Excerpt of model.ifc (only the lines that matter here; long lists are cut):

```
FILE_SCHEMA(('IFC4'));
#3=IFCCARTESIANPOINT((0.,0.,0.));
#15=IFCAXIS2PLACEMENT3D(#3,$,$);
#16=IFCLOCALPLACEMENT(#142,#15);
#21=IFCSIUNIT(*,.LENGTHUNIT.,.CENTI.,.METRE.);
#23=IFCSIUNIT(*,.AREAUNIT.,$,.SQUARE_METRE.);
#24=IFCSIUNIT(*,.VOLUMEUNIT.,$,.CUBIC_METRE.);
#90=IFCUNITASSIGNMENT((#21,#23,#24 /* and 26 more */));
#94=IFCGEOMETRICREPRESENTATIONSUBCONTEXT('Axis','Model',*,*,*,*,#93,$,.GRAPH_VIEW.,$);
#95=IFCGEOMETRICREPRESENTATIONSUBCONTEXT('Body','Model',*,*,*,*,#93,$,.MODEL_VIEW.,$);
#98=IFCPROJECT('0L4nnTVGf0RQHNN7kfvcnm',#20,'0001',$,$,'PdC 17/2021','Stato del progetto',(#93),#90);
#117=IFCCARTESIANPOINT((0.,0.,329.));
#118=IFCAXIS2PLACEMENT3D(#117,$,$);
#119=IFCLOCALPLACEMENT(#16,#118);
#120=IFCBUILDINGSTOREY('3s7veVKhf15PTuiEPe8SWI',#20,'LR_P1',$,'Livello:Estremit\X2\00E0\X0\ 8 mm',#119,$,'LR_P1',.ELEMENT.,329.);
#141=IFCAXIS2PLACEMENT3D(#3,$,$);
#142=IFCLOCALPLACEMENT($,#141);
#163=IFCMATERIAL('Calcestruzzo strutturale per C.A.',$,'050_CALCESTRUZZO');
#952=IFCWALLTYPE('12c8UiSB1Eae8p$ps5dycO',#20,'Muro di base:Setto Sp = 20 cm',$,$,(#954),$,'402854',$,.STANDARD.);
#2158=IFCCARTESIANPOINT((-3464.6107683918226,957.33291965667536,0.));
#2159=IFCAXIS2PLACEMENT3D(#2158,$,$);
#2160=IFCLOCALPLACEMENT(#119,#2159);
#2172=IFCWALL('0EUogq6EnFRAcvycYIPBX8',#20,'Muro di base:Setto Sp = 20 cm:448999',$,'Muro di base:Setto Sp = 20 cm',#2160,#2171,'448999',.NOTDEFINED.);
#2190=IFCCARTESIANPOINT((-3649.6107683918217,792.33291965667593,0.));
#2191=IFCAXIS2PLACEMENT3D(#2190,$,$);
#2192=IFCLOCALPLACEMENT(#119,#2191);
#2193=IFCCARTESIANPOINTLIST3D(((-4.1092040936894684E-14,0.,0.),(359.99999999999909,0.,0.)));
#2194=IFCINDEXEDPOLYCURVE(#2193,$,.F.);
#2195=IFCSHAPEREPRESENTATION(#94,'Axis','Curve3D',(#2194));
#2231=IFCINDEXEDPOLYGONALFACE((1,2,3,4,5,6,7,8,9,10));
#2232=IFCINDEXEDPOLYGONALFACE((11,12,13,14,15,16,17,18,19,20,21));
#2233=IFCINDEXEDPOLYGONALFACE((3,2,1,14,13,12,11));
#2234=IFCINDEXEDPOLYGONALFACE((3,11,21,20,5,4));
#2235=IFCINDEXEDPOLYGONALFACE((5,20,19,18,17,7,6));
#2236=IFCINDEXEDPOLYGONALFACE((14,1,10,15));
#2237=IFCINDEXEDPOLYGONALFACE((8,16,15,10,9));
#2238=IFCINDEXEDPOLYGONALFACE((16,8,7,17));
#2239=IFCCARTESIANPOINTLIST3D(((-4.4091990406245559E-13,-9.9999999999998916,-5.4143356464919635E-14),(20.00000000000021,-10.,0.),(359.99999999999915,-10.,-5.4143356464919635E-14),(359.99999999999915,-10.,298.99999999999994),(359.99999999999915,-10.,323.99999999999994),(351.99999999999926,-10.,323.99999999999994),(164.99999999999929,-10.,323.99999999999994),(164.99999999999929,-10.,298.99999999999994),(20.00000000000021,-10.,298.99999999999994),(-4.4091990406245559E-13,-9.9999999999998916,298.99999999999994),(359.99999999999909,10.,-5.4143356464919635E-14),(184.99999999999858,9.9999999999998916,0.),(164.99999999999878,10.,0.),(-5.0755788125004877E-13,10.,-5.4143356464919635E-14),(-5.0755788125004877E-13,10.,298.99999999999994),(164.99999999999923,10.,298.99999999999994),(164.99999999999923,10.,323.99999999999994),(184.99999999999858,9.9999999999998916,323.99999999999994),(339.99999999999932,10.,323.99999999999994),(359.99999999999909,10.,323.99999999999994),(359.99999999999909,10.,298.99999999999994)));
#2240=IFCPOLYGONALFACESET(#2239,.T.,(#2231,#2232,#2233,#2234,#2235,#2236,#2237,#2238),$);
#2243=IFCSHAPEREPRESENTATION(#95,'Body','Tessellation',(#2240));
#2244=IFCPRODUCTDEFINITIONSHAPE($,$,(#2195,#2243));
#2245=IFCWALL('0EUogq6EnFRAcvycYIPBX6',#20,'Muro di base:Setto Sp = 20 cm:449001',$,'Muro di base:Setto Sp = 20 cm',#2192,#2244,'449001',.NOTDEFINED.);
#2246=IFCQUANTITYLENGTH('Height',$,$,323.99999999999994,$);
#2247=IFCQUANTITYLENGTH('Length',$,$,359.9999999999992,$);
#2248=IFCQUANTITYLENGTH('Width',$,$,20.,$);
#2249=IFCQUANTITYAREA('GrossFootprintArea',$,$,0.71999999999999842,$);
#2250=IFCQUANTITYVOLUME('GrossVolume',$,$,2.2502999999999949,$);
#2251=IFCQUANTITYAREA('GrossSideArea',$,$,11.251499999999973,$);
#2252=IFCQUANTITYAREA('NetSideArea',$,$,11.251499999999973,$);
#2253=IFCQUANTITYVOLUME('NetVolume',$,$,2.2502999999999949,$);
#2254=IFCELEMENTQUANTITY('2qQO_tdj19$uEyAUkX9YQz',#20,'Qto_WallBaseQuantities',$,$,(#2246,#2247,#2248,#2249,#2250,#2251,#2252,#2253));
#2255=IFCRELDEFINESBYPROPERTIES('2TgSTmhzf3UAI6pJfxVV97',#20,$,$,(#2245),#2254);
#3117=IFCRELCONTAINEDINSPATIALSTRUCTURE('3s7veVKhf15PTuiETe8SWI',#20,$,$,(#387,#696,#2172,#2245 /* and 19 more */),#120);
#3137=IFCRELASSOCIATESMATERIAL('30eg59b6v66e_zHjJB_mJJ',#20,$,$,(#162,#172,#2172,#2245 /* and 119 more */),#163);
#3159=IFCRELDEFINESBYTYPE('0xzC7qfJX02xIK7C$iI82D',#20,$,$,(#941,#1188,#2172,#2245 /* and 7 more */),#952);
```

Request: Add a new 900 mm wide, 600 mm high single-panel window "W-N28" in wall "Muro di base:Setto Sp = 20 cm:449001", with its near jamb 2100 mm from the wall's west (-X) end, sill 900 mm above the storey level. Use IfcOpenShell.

```python
import numpy as np
import ifcopenshell
import ifcopenshell.api.feature
import ifcopenshell.api.geometry
import ifcopenshell.api.pset
import ifcopenshell.api.root
import ifcopenshell.api.spatial
import ifcopenshell.geom
import ifcopenshell.util.element
import ifcopenshell.util.placement
import ifcopenshell.util.representation
import ifcopenshell.util.shape
import ifcopenshell.util.unit

model = ifcopenshell.open("model.ifc")
unit_scale = ifcopenshell.util.unit.calculate_unit_scale(model)
area_scale = ifcopenshell.util.unit.calculate_unit_scale(model, "AREAUNIT")
volume_scale = ifcopenshell.util.unit.calculate_unit_scale(model, "VOLUMEUNIT")
settings = ifcopenshell.geom.settings()


def volume(element):
    """Net volume in cubic metres, openings subtracted."""
    shape = ifcopenshell.geom.create_shape(settings, element)
    return ifcopenshell.util.shape.get_volume(shape.geometry)


wall = model.by_guid("0EUogq6EnFRAcvycYIPBX6")
storey = ifcopenshell.util.element.get_container(wall, ifc_class="IfcBuildingStorey")
context = ifcopenshell.util.representation.get_context(model, "Model", "Body", "MODEL_VIEW")
before = volume(wall)

width, height, from_end, sill = 0.9, 0.6, 2.1, 0.9  # metres

# The wall runs along its own X axis, and the end named is its -X end.
wall_shape = ifcopenshell.geom.create_shape(settings, wall)
x, y, z = ifcopenshell.util.shape.get_vertices(wall_shape.geometry).T
start = x.min() + from_end
face, thickness = float(y.min()), float(y.max() - y.min())
wall_matrix = ifcopenshell.util.placement.get_local_placement(wall.ObjectPlacement)
level = ifcopenshell.util.placement.get_local_placement(storey.ObjectPlacement)[2, 3]


def in_wall(x, y):
    """Placement at x, y metres in the wall's axes, at sill height."""
    matrix = wall_matrix.copy()
    matrix[:, 3] = wall_matrix @ np.array([x / unit_scale, y / unit_scale, 0.0, 1.0])
    matrix[2, 3] = level + sill / unit_scale
    return matrix


# Opening: a box that overshoots both wall faces by 50 mm.
opening = ifcopenshell.api.root.create_entity(model, ifc_class="IfcOpeningElement", predefined_type="OPENING")
box = ifcopenshell.api.geometry.add_wall_representation(
    model, context=context, length=width, height=height, thickness=thickness + 0.1
)
ifcopenshell.api.geometry.assign_representation(model, product=opening, representation=box)
ifcopenshell.api.geometry.edit_object_placement(model, product=opening, matrix=in_wall(start, face - 0.05), is_si=False)
ifcopenshell.api.feature.add_feature(model, feature=opening, element=wall)

window = ifcopenshell.api.root.create_entity(model, ifc_class="IfcWindow", name="W-N28", predefined_type="WINDOW")
window.OverallWidth, window.OverallHeight = width / unit_scale, height / unit_scale
window.PartitioningType = "SINGLE_PANEL"
body = ifcopenshell.api.geometry.add_window_representation(
    model,
    context=context,
    overall_width=window.OverallWidth,
    overall_height=window.OverallHeight,
    partition_type="SINGLE_PANEL",
)
ifcopenshell.api.geometry.assign_representation(model, product=window, representation=body)
ifcopenshell.api.spatial.assign_container(model, products=[window], relating_structure=storey)
ifcopenshell.api.feature.add_filling(model, opening=opening, element=window)

# Centre the window in the wall's thickness.
ifcopenshell.api.geometry.edit_object_placement(model, product=window, matrix=in_wall(start, face), is_si=False)
window_shape = ifcopenshell.geom.create_shape(settings, window)
depth = ifcopenshell.util.shape.get_vertices(window_shape.geometry)[:, 1]
offset = face + thickness / 2 - (depth.min() + depth.max()) / 2
ifcopenshell.api.geometry.edit_object_placement(model, product=window, matrix=in_wall(start, offset), is_si=False)

after = volume(wall)

# Update the wall's stored quantities.
qto = model.by_id(ifcopenshell.util.element.get_pset(wall, "Qto_WallBaseQuantities", should_inherit=False)["id"])
ifcopenshell.api.pset.edit_qto(model, qto=qto, properties={
    "NetSideArea": after / thickness / area_scale,
    "NetVolume": after / volume_scale,
})

print(f"wall volume {before:.3f} -> {after:.3f} m3")

model.write("model_edited.ifc")
```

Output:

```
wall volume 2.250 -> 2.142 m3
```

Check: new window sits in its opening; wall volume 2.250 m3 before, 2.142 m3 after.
